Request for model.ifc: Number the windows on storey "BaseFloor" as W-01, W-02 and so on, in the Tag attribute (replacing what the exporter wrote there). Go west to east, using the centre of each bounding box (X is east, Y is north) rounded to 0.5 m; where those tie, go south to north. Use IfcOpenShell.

First a look at what the model holds.

```python
import ifcopenshell
import ifcopenshell.util.element
import ifcopenshell.util.placement

model = ifcopenshell.open("model.ifc")
print(model.schema)
storey = next(s for s in model.by_type("IfcBuildingStorey") if s.Name == "BaseFloor")
windows = [e for e in ifcopenshell.util.element.get_decomposition(storey) if e.is_a("IfcWindow")]
for e in sorted(windows, key=lambda e: e.id()):
    origin = ifcopenshell.util.placement.get_local_placement(e.ObjectPlacement)[:3, 3]
    print(e.id(), e.Tag, e.Name, origin.round(2) + 0.0, sep=" | ")
```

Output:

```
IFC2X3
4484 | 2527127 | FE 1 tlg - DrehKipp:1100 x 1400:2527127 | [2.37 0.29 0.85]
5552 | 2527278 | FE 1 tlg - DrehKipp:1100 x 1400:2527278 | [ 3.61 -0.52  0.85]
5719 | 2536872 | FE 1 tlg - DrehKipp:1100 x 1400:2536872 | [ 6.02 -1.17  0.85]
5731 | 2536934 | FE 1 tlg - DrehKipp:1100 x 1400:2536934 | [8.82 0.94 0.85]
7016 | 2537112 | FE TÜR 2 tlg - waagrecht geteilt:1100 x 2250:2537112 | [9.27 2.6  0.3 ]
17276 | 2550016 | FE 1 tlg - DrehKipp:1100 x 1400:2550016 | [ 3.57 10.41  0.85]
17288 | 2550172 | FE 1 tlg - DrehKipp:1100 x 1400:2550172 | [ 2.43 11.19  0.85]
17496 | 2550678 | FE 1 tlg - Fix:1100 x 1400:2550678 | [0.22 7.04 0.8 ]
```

```python
import ifcopenshell
import ifcopenshell.geom
import ifcopenshell.util.element
import ifcopenshell.util.shape

model = ifcopenshell.open("model.ifc")
settings = ifcopenshell.geom.settings()
settings.set("use-world-coords", True)


def centre(element):
    shape = ifcopenshell.geom.create_shape(settings, element)
    return ifcopenshell.util.shape.get_bbox_centroid(shape.geometry)


storey = next(s for s in model.by_type("IfcBuildingStorey") if s.Name == "BaseFloor")
windows = [e for e in ifcopenshell.util.element.get_decomposition(storey) if e.is_a("IfcWindow")]

# Insertion points can sit at a corner or the storey origin, so sort by the geometry (in metres).
centres = {e: centre(e) for e in windows}
windows.sort(key=lambda e: (round(centres[e][0] / 0.5), centres[e][1]))

for i, e in enumerate(windows, start=1):
    number = f"W-{i:02d}"
    e.Tag = number
    print(e.id(), number)

model.write("model-out.ifc")
```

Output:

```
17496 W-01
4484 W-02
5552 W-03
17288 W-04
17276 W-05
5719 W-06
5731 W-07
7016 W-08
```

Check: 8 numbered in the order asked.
